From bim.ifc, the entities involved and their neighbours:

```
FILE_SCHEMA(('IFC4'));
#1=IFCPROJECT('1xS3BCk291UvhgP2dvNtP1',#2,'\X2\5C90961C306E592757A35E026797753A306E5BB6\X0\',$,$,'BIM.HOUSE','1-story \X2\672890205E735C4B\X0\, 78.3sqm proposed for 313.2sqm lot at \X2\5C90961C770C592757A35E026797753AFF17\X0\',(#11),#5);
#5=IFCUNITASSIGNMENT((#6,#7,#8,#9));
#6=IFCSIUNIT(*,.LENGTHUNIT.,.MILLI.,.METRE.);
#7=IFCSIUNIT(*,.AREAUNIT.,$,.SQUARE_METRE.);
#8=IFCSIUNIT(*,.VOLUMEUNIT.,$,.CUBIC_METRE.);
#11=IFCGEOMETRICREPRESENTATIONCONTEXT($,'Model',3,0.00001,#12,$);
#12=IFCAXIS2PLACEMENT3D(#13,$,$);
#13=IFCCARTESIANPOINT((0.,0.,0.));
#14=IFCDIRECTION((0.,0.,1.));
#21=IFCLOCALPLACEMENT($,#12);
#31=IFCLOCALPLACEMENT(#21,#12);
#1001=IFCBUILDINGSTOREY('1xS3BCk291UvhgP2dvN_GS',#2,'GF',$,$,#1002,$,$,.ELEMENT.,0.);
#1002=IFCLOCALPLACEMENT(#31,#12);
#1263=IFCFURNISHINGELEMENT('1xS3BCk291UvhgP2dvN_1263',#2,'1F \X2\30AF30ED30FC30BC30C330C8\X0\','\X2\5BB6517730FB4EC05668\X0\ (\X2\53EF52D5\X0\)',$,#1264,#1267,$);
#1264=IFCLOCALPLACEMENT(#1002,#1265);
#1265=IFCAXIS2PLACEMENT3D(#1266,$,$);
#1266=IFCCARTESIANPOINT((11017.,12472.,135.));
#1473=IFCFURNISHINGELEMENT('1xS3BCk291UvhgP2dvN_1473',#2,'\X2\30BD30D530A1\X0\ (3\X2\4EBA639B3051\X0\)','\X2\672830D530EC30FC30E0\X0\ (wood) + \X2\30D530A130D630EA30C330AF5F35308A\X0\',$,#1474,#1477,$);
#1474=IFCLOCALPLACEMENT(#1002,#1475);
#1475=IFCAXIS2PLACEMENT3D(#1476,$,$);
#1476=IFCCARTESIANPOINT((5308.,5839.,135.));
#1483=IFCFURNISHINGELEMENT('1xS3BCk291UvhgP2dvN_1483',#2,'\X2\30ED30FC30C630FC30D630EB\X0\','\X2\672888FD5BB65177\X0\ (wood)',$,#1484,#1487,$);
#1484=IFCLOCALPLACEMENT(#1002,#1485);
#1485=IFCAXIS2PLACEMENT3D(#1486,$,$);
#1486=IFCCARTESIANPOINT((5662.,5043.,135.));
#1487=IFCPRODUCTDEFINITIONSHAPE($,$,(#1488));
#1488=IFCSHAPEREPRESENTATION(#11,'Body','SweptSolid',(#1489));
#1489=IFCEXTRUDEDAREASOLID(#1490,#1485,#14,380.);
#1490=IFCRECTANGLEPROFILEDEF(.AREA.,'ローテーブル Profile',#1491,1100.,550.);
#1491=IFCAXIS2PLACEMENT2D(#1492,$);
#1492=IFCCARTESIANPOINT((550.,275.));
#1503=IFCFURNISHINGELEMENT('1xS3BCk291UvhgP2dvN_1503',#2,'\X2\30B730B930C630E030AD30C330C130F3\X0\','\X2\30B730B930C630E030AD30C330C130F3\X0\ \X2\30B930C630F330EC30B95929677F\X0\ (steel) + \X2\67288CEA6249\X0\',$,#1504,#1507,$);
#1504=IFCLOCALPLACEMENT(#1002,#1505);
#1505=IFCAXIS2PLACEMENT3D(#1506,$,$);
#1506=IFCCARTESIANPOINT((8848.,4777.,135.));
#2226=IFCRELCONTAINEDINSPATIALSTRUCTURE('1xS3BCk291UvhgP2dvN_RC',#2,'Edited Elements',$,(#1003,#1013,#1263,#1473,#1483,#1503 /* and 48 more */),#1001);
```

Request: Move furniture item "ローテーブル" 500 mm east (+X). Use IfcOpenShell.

```python
import ifcopenshell
import ifcopenshell.api.geometry
import ifcopenshell.util.placement

model = ifcopenshell.open("bim.ifc")

item = model.by_guid("1xS3BCk291UvhgP2dvN_1483")
matrix = ifcopenshell.util.placement.get_local_placement(item.ObjectPlacement)
matrix[0, 3] += 500.0
ifcopenshell.api.geometry.edit_object_placement(model, product=item, matrix=matrix, is_si=False)

print(ifcopenshell.util.placement.get_local_placement(item.ObjectPlacement).round(3) + 0.0)

model.write("bim-out.ifc")
```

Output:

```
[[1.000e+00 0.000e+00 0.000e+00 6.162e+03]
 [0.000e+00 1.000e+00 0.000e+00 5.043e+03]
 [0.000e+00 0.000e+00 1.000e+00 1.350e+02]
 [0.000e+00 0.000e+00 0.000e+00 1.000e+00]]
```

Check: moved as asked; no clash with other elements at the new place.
